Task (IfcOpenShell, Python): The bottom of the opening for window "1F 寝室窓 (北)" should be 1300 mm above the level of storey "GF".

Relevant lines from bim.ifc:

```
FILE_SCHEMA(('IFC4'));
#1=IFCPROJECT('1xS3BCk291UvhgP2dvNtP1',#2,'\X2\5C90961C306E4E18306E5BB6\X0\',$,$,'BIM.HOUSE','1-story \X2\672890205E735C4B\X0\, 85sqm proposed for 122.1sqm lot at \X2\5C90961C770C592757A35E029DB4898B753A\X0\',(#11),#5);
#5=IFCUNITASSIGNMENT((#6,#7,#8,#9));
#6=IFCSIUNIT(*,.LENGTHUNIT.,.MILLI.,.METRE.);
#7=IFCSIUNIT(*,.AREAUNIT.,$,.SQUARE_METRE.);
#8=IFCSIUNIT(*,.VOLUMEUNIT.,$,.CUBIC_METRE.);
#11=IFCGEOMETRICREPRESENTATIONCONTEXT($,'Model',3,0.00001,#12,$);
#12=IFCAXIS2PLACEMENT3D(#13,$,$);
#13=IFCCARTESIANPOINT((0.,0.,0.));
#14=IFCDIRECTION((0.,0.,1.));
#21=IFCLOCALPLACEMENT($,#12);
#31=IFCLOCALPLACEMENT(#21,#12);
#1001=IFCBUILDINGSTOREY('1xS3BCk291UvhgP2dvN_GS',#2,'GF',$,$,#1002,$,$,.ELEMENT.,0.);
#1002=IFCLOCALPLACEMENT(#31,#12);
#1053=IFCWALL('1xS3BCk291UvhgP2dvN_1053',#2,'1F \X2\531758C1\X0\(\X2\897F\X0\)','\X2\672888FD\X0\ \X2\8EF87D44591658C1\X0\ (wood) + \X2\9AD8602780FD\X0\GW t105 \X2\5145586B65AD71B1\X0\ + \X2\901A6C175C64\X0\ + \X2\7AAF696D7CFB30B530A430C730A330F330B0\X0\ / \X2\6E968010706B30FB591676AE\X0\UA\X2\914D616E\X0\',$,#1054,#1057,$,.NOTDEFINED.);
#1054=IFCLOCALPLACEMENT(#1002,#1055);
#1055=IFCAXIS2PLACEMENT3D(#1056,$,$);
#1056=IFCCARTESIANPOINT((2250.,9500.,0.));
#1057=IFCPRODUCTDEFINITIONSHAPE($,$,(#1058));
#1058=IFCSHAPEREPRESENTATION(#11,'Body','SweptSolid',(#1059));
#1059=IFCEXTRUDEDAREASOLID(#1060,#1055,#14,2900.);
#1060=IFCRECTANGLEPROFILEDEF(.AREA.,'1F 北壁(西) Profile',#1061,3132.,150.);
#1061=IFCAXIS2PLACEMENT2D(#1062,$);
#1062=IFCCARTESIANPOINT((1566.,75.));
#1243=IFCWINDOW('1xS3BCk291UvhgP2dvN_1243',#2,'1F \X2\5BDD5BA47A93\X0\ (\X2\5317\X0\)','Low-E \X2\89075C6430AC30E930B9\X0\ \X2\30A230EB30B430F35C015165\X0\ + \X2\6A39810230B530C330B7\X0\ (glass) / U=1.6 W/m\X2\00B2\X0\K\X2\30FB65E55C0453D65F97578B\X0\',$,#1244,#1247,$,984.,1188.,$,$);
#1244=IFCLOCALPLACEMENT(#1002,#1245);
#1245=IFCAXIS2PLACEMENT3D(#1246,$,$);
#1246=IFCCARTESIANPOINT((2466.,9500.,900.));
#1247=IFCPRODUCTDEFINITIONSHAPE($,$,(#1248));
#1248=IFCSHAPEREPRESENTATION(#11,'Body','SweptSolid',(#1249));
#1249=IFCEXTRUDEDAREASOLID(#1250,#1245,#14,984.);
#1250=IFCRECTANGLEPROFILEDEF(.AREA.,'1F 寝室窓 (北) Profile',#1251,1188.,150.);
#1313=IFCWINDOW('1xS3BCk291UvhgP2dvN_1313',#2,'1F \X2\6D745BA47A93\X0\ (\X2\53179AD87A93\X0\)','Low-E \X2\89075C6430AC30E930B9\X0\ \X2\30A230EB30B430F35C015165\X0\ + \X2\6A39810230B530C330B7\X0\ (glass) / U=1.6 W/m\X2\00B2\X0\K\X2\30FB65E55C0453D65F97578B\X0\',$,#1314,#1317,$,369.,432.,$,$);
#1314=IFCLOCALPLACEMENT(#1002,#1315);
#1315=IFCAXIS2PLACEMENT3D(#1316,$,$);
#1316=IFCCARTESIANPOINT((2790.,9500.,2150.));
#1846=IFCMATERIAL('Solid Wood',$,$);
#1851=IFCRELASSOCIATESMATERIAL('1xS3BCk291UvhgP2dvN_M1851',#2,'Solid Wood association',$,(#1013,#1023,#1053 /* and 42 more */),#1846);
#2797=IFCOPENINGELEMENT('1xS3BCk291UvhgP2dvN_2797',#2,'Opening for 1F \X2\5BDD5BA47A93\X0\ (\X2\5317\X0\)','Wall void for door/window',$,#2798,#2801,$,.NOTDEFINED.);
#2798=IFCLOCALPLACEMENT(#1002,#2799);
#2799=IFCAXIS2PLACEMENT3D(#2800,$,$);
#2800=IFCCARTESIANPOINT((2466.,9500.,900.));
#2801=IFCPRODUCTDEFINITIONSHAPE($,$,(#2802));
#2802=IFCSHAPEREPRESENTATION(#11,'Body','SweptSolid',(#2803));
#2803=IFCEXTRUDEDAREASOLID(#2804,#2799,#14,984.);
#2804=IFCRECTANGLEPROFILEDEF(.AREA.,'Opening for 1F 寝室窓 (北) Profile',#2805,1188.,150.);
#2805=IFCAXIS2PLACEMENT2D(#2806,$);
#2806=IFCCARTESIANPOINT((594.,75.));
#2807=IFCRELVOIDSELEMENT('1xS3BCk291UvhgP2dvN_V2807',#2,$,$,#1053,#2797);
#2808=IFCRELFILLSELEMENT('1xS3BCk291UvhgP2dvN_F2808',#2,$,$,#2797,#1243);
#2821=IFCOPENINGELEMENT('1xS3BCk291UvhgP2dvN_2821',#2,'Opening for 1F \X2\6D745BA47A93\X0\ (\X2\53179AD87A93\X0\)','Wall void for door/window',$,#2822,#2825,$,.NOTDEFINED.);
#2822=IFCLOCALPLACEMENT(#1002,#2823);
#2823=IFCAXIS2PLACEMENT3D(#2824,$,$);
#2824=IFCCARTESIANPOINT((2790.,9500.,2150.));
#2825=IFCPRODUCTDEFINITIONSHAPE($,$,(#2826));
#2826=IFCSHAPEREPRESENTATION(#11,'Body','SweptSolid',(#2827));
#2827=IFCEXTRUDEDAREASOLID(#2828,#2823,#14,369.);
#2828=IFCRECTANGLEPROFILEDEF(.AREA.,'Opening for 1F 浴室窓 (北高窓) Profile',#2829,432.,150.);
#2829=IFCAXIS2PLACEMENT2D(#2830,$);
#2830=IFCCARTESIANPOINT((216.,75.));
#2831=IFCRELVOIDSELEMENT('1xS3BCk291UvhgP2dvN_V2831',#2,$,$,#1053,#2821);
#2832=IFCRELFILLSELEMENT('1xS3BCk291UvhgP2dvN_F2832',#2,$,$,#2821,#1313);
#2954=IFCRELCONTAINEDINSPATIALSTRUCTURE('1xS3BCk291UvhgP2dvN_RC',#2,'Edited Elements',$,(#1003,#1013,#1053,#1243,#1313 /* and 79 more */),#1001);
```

```python
import numpy as np
import ifcopenshell
import ifcopenshell.api.geometry
import ifcopenshell.geom
import ifcopenshell.util.element
import ifcopenshell.util.placement
import ifcopenshell.util.shape
import ifcopenshell.util.unit

model = ifcopenshell.open("bim.ifc")
unit_scale = ifcopenshell.util.unit.calculate_unit_scale(model)

window = model.by_guid("1xS3BCk291UvhgP2dvN_1243")
opening = window.FillsVoids[0].RelatingOpeningElement
storey = ifcopenshell.util.element.get_container(window, ifc_class="IfcBuildingStorey")
level = ifcopenshell.util.placement.get_local_placement(storey.ObjectPlacement)[2, 3]

# The opening's origin need not be at the sill, so measure its lowest point.
shape = ifcopenshell.geom.create_shape(ifcopenshell.geom.settings(), opening)
bottom = ifcopenshell.util.shape.get_shape_bottom_elevation(shape, shape.geometry) / unit_scale
dz = level + 1300.0 - bottom

shift = np.array([0.0, 0.0, dz])
# The window is not placed relative to its opening, so move both.
for product in (opening, window):
    matrix = ifcopenshell.util.placement.get_local_placement(product.ObjectPlacement)
    matrix[:3, 3] += shift
    ifcopenshell.api.geometry.edit_object_placement(model, product=product, matrix=matrix, is_si=False)

print(f"moved by {dz * unit_scale:+.3f} m")

model.write("bim_v2.ifc")
```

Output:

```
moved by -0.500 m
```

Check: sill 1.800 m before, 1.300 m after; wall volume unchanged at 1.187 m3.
